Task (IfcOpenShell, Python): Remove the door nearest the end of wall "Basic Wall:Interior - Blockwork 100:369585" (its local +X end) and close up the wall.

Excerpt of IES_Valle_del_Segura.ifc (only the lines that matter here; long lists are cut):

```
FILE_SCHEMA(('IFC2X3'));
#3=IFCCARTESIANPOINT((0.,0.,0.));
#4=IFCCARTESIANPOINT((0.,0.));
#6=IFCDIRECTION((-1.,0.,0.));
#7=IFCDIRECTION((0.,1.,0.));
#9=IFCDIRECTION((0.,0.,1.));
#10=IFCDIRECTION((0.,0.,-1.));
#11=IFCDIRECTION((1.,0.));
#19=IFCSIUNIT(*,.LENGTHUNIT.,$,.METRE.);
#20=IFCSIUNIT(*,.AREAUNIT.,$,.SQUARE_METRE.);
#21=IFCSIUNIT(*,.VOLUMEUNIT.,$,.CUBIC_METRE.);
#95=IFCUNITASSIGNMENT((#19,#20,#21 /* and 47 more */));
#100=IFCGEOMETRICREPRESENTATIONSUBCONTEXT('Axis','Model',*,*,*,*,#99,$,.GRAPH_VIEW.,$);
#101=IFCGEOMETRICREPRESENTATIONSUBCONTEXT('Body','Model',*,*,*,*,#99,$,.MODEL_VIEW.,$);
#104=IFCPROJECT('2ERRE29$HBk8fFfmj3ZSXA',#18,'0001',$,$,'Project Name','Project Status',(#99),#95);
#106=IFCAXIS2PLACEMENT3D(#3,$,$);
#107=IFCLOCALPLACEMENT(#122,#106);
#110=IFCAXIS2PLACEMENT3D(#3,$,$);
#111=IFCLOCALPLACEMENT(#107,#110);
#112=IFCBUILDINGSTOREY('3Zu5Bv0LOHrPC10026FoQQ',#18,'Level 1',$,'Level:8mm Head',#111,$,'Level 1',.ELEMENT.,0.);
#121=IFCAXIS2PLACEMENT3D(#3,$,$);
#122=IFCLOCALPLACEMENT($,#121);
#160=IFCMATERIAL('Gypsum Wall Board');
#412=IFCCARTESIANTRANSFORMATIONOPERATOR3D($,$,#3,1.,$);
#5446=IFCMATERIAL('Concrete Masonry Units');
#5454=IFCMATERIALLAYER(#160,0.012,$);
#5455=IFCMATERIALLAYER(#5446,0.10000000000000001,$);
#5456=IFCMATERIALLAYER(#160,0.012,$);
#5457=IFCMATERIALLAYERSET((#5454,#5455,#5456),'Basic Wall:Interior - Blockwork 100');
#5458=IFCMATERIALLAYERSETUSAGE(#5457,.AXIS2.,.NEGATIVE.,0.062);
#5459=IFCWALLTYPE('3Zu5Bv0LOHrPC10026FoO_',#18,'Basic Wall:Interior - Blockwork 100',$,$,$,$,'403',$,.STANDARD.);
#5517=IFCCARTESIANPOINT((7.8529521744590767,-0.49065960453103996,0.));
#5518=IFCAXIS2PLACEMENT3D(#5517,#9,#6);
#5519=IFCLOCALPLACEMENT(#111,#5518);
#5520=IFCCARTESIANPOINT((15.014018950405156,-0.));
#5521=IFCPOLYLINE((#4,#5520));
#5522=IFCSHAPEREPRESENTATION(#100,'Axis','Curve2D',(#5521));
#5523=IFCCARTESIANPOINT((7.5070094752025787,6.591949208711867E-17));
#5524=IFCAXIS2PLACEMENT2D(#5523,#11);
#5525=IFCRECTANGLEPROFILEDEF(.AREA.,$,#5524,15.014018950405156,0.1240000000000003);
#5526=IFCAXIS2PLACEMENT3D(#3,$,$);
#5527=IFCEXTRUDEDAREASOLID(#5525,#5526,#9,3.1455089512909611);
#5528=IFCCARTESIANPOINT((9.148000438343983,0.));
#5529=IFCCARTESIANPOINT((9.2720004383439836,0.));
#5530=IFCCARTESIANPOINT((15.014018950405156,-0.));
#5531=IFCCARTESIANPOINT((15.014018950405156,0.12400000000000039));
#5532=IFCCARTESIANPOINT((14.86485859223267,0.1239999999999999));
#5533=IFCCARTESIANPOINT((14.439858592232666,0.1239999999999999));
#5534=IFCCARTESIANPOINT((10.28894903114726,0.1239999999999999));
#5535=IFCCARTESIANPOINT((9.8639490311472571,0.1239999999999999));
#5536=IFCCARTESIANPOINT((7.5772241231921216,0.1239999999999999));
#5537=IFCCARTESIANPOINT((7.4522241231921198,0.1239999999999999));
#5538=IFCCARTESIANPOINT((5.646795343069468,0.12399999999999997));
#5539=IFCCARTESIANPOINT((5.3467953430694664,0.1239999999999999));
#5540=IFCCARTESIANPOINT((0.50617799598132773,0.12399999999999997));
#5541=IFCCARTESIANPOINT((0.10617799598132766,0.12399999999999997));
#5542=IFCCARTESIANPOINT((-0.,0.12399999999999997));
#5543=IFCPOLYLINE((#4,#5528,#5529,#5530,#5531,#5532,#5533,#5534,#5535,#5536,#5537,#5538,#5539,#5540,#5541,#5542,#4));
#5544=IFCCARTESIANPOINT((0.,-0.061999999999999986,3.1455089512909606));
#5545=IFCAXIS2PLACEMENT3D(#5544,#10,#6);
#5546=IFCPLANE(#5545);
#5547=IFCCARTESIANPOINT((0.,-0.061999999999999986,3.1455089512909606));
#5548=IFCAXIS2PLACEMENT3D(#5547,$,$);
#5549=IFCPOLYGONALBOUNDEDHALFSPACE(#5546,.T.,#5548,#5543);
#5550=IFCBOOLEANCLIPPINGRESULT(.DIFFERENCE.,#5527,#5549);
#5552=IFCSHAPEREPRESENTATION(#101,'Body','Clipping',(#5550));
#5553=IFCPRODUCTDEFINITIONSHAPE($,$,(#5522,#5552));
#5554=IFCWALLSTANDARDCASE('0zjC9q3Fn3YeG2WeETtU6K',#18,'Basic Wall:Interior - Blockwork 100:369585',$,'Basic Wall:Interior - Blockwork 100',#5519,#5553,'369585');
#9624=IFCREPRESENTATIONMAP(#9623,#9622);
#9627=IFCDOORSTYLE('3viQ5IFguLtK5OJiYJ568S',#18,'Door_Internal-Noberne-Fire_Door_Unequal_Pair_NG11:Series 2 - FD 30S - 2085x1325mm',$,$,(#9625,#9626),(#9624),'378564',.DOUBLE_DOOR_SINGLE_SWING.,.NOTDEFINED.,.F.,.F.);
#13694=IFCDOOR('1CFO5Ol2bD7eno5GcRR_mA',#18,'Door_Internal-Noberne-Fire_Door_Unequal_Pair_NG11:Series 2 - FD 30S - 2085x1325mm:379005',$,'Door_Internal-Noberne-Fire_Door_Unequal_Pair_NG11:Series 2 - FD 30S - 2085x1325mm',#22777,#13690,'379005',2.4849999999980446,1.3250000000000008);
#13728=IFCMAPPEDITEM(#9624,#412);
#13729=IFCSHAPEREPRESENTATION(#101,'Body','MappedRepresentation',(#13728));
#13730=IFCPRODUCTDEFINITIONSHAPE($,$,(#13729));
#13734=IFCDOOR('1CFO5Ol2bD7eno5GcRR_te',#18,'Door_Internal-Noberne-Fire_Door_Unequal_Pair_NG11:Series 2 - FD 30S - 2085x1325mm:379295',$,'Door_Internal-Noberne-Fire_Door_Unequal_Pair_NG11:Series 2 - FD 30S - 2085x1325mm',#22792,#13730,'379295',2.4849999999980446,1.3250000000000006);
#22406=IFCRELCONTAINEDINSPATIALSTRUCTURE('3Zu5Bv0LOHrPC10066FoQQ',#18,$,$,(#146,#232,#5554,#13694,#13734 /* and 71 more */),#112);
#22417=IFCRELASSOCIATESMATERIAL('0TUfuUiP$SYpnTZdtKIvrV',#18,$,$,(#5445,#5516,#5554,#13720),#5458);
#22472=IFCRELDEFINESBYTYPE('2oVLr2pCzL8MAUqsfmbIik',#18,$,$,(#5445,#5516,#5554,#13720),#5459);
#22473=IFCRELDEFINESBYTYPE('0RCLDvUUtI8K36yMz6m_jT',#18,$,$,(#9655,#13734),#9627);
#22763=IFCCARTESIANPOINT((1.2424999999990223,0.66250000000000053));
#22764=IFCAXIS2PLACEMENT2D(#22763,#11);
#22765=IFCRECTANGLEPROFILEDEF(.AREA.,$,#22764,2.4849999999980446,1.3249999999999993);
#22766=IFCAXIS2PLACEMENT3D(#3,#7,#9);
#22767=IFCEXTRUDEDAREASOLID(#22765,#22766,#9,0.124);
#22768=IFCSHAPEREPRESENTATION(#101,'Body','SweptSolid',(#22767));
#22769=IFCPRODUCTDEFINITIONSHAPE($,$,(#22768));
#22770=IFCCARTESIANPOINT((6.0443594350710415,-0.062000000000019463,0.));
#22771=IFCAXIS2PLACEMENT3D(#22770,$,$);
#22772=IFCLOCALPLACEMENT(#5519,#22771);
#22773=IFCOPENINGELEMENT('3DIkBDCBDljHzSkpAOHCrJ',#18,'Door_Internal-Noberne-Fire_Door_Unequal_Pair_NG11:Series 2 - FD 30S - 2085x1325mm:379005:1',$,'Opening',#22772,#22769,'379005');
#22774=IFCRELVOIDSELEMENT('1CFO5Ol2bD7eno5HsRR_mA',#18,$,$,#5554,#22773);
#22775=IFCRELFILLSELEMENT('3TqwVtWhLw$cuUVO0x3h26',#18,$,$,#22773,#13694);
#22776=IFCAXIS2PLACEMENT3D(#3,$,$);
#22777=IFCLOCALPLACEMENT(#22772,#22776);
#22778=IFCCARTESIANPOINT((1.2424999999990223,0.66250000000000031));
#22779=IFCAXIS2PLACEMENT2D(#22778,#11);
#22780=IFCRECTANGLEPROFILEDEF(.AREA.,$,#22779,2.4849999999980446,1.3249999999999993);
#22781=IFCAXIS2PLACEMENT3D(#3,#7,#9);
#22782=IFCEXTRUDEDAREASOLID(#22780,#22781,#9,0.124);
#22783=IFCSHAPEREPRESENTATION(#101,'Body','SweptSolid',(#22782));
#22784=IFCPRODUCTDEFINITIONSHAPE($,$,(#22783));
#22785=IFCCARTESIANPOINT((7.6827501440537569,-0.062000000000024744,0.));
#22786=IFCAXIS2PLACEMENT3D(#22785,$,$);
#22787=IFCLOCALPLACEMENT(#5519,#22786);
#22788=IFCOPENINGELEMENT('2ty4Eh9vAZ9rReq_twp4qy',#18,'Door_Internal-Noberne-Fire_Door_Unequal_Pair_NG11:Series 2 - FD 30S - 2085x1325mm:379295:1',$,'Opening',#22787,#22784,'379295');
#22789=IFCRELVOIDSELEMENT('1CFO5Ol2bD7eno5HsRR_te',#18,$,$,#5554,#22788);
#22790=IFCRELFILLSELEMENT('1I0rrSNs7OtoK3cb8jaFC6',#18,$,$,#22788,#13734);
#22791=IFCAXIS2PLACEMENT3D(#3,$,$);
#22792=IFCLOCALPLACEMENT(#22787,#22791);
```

```python
import ifcopenshell
import ifcopenshell.api.feature
import ifcopenshell.api.root
import ifcopenshell.geom
import ifcopenshell.util.shape

model = ifcopenshell.open("IES_Valle_del_Segura.ifc")
settings = ifcopenshell.geom.settings()


def volume(element):
    """Net volume in cubic metres, openings subtracted."""
    shape = ifcopenshell.geom.create_shape(settings, element)
    return ifcopenshell.util.shape.get_volume(shape.geometry)


door = model.by_guid("1CFO5Ol2bD7eno5GcRR_te")
opening = door.FillsVoids[0].RelatingOpeningElement
wall = opening.VoidsElements[0].RelatingBuildingElement
before = volume(wall)

ifcopenshell.api.root.remove_product(model, product=door)
ifcopenshell.api.feature.remove_feature(model, feature=opening)

after = volume(wall)

print(f"wall volume {before:.3f} -> {after:.3f} m3")

model.write("IES_Valle_del_Segura_rev.ifc")
```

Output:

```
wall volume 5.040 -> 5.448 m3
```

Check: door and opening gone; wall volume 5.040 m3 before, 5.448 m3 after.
